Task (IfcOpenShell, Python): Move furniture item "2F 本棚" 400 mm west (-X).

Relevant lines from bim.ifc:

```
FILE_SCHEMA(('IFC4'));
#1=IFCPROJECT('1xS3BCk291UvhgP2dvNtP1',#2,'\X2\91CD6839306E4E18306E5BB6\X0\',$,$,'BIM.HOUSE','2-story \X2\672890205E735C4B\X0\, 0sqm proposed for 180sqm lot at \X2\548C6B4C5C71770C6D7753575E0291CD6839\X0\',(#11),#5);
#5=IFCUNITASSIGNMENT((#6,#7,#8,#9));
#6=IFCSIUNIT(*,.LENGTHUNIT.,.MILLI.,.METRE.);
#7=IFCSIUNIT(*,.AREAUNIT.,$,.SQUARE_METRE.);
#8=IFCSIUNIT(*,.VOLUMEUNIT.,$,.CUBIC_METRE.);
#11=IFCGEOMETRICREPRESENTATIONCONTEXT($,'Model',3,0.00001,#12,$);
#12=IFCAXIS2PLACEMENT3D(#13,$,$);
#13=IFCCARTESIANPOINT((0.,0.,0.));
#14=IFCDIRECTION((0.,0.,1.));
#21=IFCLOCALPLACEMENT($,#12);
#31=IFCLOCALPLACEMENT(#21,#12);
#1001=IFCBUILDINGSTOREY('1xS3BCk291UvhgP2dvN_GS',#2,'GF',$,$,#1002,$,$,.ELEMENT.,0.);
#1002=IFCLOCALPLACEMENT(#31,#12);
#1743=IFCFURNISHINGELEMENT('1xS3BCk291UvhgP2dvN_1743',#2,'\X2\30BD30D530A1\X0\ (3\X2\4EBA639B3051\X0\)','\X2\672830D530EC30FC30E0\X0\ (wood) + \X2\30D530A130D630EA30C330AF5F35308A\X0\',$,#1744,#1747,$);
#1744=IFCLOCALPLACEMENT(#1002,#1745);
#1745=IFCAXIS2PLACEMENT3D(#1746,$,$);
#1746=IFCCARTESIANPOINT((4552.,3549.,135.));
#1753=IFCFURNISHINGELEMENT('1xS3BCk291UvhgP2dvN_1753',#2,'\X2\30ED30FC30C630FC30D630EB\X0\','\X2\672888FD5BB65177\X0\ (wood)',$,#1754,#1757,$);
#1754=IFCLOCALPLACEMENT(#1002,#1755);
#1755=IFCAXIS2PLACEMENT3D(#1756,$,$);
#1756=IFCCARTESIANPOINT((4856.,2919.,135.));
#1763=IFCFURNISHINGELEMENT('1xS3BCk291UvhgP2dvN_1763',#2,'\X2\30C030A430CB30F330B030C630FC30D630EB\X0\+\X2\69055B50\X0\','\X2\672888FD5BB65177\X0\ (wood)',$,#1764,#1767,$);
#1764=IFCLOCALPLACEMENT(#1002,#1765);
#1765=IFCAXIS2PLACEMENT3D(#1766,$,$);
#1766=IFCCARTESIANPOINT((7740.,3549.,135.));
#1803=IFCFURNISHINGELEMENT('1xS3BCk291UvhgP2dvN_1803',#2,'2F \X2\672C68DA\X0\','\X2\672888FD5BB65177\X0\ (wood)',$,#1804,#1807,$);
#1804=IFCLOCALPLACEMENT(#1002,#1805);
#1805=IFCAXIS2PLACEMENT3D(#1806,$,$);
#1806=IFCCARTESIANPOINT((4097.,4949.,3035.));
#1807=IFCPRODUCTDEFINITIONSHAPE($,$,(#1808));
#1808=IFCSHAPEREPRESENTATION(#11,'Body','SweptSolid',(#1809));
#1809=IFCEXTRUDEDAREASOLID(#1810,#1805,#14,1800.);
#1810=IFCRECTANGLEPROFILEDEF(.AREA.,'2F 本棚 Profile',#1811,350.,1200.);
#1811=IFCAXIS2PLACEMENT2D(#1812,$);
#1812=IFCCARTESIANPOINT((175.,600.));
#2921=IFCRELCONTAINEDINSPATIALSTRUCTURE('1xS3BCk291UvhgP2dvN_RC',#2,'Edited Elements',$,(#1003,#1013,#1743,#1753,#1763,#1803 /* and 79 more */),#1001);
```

```python
import ifcopenshell
import ifcopenshell.api.geometry
import ifcopenshell.util.placement
import ifcopenshell.util.unit

model = ifcopenshell.open("bim.ifc")
unit_scale = ifcopenshell.util.unit.calculate_unit_scale(model)

item = model.by_id(1803)
matrix = ifcopenshell.util.placement.get_local_placement(item.ObjectPlacement)
matrix[0, 3] -= 0.4 / unit_scale
ifcopenshell.api.geometry.edit_object_placement(model, product=item, matrix=matrix, is_si=False)

print(ifcopenshell.util.placement.get_local_placement(item.ObjectPlacement).round(3) + 0.0)

model.write("bim_updated.ifc")
```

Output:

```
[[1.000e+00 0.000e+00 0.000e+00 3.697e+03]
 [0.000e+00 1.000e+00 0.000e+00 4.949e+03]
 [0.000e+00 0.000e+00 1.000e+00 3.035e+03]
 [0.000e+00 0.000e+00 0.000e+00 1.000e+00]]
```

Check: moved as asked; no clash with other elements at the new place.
